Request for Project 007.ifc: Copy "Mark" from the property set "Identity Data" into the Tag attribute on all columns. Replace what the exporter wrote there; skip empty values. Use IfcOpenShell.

First a look at what the model holds.

```python
import ifcopenshell
import ifcopenshell.util.element

model = ifcopenshell.open("Project 007.ifc")
print(model.schema)
columns = model.by_type("IfcColumn")
print(len(columns), "columns")
for e in columns[:8]:
    source = ifcopenshell.util.element.get_pset(e, "Identity Data", "Mark")
    target = e.Tag
    print(e.id(), repr(source), repr(target), sep=" | ")
```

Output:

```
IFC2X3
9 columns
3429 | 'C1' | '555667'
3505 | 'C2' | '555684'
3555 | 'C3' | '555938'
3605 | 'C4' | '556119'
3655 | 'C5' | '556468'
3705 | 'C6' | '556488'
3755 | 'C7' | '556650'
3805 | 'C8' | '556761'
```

```python
import ifcopenshell
import ifcopenshell.util.element

model = ifcopenshell.open("Project 007.ifc")

count = 0
for e in model.by_type("IfcColumn"):
    value = ifcopenshell.util.element.get_pset(e, "Identity Data", "Mark")
    current = e.Tag
    if not value or not value.strip() or current == value:
        continue
    e.Tag = value
    count += 1

print(count, "columns updated")

model.write("Project 007-out.ifc")
```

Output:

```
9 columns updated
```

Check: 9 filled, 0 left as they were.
